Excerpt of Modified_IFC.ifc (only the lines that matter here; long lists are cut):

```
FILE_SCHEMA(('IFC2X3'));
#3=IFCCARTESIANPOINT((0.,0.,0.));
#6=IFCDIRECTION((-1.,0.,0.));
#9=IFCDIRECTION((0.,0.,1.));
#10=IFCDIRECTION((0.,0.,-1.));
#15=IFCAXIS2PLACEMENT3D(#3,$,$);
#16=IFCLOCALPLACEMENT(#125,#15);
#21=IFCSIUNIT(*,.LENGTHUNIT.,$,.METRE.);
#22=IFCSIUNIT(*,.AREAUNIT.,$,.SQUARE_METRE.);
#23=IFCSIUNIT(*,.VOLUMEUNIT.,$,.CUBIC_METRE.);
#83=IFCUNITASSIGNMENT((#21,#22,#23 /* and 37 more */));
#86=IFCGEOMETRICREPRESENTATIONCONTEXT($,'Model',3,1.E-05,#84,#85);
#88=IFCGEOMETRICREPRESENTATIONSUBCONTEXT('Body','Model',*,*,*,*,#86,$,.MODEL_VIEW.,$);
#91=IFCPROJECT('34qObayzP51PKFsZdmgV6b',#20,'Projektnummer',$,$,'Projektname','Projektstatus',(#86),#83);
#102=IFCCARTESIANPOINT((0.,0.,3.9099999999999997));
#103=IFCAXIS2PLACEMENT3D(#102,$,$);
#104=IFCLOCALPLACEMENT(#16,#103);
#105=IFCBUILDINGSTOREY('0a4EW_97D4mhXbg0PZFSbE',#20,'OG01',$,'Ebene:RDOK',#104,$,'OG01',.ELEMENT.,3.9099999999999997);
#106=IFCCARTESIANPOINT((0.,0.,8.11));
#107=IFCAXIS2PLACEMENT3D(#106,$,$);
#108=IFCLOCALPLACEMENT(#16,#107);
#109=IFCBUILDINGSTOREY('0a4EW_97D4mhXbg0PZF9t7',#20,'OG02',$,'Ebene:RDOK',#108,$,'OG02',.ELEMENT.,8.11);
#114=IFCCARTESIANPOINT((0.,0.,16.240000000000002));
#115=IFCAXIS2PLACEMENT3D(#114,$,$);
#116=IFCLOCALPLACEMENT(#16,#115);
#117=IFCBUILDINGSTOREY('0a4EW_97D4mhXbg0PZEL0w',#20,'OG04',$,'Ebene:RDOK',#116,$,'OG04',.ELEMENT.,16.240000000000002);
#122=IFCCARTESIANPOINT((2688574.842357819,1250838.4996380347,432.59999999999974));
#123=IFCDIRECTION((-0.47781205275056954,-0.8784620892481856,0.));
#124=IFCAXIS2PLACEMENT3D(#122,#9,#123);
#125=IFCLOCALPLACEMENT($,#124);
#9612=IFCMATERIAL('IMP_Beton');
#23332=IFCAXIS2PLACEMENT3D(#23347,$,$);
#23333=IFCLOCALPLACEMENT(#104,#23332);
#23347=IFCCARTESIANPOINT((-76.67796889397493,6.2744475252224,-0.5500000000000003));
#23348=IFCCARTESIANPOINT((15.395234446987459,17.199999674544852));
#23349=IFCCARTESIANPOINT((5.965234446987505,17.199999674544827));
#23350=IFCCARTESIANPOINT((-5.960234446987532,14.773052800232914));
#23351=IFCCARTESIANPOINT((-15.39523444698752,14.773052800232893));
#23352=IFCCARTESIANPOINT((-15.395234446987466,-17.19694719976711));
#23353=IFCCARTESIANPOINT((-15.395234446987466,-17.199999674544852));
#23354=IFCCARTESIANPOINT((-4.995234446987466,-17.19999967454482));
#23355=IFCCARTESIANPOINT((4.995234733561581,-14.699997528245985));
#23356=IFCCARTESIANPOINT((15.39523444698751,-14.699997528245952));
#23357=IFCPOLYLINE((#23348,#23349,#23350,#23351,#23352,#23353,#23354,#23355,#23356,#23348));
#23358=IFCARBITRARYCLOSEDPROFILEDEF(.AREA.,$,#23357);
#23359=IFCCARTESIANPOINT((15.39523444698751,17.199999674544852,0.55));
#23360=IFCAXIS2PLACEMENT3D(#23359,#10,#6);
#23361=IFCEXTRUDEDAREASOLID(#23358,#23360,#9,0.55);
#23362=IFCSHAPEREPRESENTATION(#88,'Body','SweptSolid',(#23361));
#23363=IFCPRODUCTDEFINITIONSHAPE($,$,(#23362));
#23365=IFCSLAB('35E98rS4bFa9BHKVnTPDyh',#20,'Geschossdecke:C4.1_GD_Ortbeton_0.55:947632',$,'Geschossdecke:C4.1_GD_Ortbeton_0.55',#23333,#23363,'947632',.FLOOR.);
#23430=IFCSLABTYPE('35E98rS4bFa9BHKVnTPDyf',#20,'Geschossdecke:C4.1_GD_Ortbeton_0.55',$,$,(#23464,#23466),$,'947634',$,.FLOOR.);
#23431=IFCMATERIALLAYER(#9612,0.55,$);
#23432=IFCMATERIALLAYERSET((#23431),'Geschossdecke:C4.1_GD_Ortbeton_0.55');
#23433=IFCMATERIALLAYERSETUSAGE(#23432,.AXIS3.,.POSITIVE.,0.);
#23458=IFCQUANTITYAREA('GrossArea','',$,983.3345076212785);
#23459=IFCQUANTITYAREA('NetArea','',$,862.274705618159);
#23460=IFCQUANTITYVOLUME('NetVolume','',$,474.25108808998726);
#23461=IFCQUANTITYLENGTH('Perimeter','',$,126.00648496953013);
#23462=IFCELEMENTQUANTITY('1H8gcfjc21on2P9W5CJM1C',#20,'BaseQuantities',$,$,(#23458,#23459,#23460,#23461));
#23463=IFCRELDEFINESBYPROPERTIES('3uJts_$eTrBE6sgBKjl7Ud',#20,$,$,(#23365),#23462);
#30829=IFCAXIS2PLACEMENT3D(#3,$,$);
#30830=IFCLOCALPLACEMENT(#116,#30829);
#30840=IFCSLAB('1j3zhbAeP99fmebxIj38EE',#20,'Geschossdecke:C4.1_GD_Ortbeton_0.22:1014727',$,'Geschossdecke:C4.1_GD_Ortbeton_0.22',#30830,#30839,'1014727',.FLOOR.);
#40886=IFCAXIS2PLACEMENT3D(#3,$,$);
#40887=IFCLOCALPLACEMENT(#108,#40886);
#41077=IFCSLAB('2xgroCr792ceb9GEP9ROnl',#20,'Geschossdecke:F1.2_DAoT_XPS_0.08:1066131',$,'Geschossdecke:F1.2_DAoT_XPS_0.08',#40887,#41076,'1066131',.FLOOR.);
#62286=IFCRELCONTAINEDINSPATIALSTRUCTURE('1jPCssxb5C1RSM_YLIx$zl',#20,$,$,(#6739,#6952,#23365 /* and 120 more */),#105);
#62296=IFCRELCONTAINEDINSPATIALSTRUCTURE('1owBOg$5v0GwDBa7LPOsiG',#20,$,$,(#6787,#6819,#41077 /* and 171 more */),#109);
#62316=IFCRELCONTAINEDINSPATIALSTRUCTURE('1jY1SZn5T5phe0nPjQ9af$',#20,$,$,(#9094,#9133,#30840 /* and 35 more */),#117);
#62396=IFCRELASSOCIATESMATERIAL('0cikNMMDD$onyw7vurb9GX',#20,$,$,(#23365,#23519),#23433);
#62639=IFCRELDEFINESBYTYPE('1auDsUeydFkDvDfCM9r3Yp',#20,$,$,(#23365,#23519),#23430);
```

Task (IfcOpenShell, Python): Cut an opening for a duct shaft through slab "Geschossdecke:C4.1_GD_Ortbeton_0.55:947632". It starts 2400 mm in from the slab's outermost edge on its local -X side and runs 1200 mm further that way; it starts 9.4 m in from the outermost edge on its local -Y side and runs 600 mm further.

```python
import numpy as np
import ifcopenshell
import ifcopenshell.api.feature
import ifcopenshell.api.geometry
import ifcopenshell.api.pset
import ifcopenshell.api.root
import ifcopenshell.geom
import ifcopenshell.util.element
import ifcopenshell.util.placement
import ifcopenshell.util.representation
import ifcopenshell.util.shape
import ifcopenshell.util.unit

model = ifcopenshell.open("Modified_IFC.ifc")
unit_scale = ifcopenshell.util.unit.calculate_unit_scale(model)
area_scale = ifcopenshell.util.unit.calculate_unit_scale(model, "AREAUNIT")
volume_scale = ifcopenshell.util.unit.calculate_unit_scale(model, "VOLUMEUNIT")
settings = ifcopenshell.geom.settings()


def volume(element):
    """Net volume in cubic metres, openings subtracted."""
    shape = ifcopenshell.geom.create_shape(settings, element)
    return ifcopenshell.util.shape.get_volume(shape.geometry)


slab = model.by_guid("35E98rS4bFa9BHKVnTPDyh")
before = volume(slab)

# Extent in the slab's own axes, in metres. The edges named are its -X and -Y sides.
slab_shape = ifcopenshell.geom.create_shape(settings, slab)
vertices = ifcopenshell.util.shape.get_vertices(slab_shape.geometry)
x_min, y_min, bottom = vertices.min(axis=0)
top = vertices[:, 2].max()

opening = ifcopenshell.api.root.create_entity(model, ifc_class="IfcOpeningElement", name="Duct shaft opening")
context = ifcopenshell.util.representation.get_context(model, "Model", "Body", "MODEL_VIEW")
width, depth = 1.2, 0.6
outline = [(0.0, 0.0), (width, 0.0), (width, depth), (0.0, depth), (0.0, 0.0)]
# Overshoot both faces by 50 mm so the cut is clean.
shape = ifcopenshell.api.geometry.add_slab_representation(
    model, context=context, depth=top - bottom + 0.1, polyline=outline
)
ifcopenshell.api.geometry.assign_representation(model, product=opening, representation=shape)

matrix = ifcopenshell.util.placement.get_local_placement(slab.ObjectPlacement)
matrix[:, 3] = matrix @ np.append(np.array([x_min + 2.4, y_min + 9.4, bottom - 0.05]) / unit_scale, 1.0)
ifcopenshell.api.geometry.edit_object_placement(model, product=opening, matrix=matrix, is_si=False)
ifcopenshell.api.feature.add_feature(model, feature=opening, element=slab)

after = volume(slab)

# Update the slab's stored quantities.
qto = model.by_id(ifcopenshell.util.element.get_pset(slab, "BaseQuantities", should_inherit=False)["id"])
ifcopenshell.api.pset.edit_qto(model, qto=qto, properties={
    "NetArea": after / (top - bottom) / area_scale,
    "NetVolume": after / volume_scale,
})

print(f"slab volume {before:.3f} -> {after:.3f} m3")

model.write("Modified_IFC_rev.ifc")
```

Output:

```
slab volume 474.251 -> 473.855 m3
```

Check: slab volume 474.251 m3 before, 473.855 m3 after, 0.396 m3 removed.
